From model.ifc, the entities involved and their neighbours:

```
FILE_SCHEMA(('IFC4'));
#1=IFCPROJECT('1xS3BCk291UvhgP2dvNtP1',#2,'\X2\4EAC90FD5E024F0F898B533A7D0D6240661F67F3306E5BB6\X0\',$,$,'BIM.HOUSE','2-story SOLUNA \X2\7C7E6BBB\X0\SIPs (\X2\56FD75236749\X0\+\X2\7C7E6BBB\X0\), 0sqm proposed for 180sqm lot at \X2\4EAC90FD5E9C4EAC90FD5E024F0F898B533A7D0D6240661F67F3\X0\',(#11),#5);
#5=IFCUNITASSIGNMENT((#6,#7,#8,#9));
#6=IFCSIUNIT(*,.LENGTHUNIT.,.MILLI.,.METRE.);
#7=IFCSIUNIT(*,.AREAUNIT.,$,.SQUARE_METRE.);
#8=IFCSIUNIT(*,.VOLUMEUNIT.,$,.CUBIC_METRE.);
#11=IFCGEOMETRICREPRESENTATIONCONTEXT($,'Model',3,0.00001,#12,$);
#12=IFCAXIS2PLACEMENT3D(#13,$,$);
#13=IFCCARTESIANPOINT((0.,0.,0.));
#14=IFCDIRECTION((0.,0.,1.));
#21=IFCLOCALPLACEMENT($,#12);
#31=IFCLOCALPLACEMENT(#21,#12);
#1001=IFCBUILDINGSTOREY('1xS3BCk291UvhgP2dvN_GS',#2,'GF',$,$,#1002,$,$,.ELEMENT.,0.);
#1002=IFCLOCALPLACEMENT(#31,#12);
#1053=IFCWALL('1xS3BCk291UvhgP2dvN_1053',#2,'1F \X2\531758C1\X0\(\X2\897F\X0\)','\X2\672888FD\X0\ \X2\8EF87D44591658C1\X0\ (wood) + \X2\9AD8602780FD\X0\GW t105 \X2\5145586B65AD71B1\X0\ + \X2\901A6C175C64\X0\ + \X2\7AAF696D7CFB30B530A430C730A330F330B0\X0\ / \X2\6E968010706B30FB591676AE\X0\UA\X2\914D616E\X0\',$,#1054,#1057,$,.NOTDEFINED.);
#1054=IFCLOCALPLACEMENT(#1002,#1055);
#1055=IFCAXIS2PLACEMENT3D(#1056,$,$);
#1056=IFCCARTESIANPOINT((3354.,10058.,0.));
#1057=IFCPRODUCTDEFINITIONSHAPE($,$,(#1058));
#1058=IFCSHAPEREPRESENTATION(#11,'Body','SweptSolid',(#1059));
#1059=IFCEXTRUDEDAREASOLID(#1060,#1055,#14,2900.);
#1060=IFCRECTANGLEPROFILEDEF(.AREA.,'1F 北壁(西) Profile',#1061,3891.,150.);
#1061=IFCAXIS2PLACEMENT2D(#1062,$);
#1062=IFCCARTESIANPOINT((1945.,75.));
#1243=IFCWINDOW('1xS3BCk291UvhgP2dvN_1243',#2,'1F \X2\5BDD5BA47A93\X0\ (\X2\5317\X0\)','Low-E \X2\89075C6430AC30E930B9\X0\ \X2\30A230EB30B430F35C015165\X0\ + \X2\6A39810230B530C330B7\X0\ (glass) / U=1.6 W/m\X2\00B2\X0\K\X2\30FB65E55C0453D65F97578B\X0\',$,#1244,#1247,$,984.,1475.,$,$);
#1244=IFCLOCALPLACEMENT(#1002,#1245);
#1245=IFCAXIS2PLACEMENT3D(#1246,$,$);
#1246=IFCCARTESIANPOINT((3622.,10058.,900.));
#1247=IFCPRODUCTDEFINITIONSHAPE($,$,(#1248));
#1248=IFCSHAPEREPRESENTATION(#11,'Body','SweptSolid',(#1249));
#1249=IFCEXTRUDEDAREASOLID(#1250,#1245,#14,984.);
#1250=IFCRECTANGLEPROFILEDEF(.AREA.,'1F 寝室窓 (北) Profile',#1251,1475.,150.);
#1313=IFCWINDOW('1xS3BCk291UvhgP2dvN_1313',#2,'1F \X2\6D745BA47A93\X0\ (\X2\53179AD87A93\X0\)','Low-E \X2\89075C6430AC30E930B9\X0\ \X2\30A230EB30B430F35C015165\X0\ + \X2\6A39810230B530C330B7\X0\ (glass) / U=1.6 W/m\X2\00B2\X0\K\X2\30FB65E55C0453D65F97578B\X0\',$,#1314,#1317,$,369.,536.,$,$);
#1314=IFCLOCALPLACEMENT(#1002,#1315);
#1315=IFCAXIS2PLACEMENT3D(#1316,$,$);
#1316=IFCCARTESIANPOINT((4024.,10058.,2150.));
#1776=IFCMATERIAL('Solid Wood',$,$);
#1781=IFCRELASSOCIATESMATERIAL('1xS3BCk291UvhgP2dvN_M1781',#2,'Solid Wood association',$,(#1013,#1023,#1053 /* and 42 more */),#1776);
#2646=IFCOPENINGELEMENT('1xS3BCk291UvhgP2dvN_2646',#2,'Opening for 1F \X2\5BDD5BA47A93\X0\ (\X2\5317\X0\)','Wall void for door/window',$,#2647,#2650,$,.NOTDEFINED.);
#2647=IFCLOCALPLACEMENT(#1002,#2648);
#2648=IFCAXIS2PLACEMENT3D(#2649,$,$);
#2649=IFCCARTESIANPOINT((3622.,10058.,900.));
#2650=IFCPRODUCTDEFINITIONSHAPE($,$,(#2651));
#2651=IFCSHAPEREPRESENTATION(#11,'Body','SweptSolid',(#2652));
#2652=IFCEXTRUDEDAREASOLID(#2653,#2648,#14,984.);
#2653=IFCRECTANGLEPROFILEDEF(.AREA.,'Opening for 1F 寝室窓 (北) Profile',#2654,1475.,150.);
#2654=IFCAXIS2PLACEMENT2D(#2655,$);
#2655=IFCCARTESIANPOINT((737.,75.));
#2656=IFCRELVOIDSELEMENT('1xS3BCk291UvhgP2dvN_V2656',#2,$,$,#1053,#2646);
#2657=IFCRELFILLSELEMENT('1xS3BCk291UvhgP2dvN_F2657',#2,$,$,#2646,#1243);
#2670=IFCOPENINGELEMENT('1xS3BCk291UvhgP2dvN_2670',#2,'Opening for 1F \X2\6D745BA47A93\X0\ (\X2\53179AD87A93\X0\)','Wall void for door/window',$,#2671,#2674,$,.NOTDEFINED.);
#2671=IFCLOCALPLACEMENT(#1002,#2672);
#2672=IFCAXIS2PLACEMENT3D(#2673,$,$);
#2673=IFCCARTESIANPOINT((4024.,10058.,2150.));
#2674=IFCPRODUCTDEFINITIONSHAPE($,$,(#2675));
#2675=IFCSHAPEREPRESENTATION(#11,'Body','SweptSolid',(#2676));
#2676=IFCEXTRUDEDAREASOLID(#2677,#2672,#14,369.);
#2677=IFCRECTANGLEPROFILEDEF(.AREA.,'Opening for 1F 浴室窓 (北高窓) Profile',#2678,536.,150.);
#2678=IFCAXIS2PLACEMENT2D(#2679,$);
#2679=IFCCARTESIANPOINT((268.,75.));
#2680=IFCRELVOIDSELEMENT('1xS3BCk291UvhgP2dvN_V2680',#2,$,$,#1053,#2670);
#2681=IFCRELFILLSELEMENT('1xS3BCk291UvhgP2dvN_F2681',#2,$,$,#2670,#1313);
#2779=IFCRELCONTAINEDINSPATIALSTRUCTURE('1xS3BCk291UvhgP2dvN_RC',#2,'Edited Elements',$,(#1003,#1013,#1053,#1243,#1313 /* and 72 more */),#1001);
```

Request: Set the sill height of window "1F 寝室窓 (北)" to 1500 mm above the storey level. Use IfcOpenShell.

```python
import numpy as np
import ifcopenshell
import ifcopenshell.api.geometry
import ifcopenshell.geom
import ifcopenshell.util.element
import ifcopenshell.util.placement
import ifcopenshell.util.shape
import ifcopenshell.util.unit

model = ifcopenshell.open("model.ifc")
unit_scale = ifcopenshell.util.unit.calculate_unit_scale(model)

window = model.by_guid("1xS3BCk291UvhgP2dvN_1243")
opening = window.FillsVoids[0].RelatingOpeningElement
storey = ifcopenshell.util.element.get_container(window, ifc_class="IfcBuildingStorey")
level = ifcopenshell.util.placement.get_local_placement(storey.ObjectPlacement)[2, 3]

# The opening's origin need not be at the sill, so measure its lowest point.
shape = ifcopenshell.geom.create_shape(ifcopenshell.geom.settings(), opening)
bottom = ifcopenshell.util.shape.get_shape_bottom_elevation(shape, shape.geometry) / unit_scale
dz = level + 1500.0 - bottom

shift = np.array([0.0, 0.0, dz])
# The window is not placed relative to its opening, so move both.
for product in (opening, window):
    matrix = ifcopenshell.util.placement.get_local_placement(product.ObjectPlacement)
    matrix[:3, 3] += shift
    ifcopenshell.api.geometry.edit_object_placement(model, product=product, matrix=matrix, is_si=False)

print(f"moved by {dz * unit_scale:+.3f} m")

model.write("model_updated.ifc")
```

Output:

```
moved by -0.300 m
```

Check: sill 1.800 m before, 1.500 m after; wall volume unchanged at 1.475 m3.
